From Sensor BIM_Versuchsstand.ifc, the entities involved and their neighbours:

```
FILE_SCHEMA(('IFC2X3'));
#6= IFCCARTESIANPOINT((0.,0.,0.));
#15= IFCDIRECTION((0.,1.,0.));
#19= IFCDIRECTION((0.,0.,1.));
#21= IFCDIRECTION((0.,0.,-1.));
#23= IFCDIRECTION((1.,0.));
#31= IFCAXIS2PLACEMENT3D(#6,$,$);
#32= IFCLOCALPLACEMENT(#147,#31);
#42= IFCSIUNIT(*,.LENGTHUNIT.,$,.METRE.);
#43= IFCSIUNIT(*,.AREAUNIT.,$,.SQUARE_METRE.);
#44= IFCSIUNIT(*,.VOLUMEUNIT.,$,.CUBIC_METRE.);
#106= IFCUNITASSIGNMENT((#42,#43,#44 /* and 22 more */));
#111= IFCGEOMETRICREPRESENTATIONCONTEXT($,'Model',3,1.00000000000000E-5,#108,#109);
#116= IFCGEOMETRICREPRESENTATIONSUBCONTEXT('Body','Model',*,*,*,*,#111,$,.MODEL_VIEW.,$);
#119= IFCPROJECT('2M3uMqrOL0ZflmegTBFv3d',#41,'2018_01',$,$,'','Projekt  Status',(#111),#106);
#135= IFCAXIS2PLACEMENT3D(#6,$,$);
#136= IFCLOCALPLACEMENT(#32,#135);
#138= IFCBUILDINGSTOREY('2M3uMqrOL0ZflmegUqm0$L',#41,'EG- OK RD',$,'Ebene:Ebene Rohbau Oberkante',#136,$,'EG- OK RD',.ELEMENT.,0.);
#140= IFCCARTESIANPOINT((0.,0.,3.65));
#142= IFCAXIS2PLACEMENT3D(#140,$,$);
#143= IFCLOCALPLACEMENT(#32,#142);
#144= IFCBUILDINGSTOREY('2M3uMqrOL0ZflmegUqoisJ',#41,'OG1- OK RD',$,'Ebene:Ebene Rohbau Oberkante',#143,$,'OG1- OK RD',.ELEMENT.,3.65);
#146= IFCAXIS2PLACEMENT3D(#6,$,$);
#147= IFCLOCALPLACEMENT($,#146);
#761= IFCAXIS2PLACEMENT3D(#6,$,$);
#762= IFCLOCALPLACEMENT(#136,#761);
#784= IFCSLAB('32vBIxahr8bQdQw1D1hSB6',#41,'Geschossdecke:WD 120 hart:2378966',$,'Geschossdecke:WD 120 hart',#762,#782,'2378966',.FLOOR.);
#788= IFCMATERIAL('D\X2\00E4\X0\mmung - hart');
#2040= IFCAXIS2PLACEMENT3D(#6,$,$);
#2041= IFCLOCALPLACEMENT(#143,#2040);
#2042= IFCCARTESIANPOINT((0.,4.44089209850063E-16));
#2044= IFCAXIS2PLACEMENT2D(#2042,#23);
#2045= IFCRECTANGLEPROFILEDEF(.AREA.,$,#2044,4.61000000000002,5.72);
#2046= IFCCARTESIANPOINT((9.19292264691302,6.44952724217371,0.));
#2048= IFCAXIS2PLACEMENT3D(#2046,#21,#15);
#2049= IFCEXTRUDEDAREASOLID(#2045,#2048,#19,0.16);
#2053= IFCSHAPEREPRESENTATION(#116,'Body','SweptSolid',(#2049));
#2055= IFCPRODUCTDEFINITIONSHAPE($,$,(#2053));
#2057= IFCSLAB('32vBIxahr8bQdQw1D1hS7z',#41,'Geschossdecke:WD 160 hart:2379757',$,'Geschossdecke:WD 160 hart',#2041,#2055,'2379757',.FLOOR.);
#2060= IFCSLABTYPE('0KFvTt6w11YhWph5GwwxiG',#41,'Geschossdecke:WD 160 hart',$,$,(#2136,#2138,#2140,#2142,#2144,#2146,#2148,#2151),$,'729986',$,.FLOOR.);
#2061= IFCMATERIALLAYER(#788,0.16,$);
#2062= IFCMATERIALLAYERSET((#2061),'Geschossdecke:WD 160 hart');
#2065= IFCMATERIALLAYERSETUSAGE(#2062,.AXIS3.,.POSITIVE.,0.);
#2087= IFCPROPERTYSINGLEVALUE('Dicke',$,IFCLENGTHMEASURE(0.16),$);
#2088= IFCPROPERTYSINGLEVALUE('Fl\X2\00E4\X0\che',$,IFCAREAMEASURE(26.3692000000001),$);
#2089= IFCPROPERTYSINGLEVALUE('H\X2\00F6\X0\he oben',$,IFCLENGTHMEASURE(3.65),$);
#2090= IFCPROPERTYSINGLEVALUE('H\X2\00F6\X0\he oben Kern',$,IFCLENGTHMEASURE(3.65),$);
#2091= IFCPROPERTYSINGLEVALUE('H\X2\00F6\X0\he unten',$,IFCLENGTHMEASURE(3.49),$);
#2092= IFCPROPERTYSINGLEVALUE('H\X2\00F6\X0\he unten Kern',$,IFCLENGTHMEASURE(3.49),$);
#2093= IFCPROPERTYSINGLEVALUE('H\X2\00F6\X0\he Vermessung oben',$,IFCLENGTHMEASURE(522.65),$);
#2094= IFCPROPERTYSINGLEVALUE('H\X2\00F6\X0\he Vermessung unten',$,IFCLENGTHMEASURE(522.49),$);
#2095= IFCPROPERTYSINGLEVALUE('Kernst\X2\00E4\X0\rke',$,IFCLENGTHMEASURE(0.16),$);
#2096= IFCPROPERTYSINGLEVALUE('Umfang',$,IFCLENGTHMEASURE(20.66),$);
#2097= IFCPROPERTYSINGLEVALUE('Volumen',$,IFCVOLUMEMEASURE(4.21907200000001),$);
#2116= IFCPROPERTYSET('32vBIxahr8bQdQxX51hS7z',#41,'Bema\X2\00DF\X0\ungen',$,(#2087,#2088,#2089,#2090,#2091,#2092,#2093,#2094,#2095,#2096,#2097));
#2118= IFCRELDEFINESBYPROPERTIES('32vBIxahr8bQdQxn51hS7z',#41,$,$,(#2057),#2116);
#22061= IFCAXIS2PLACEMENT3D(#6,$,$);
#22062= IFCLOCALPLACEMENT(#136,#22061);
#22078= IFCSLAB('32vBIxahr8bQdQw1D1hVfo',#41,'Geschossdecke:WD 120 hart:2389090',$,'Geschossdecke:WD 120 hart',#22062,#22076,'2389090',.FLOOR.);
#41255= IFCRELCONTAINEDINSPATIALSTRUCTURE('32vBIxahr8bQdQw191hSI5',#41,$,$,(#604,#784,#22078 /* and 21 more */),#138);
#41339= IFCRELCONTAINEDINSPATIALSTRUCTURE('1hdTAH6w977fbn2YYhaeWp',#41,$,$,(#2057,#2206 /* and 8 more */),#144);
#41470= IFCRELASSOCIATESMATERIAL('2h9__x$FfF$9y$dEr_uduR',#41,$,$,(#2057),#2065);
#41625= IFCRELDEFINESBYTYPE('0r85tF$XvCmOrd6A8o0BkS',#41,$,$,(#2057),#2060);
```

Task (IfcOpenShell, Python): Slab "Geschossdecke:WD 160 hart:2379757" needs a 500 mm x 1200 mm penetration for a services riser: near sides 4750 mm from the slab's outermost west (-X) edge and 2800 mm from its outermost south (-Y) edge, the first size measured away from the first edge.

```python
import numpy as np
import ifcopenshell
import ifcopenshell.api.feature
import ifcopenshell.api.geometry
import ifcopenshell.api.pset
import ifcopenshell.api.root
import ifcopenshell.geom
import ifcopenshell.util.element
import ifcopenshell.util.placement
import ifcopenshell.util.representation
import ifcopenshell.util.shape
import ifcopenshell.util.unit

model = ifcopenshell.open("Sensor BIM_Versuchsstand.ifc")
unit_scale = ifcopenshell.util.unit.calculate_unit_scale(model)
area_scale = ifcopenshell.util.unit.calculate_unit_scale(model, "AREAUNIT")
volume_scale = ifcopenshell.util.unit.calculate_unit_scale(model, "VOLUMEUNIT")
settings = ifcopenshell.geom.settings()


def volume(element):
    """Net volume in cubic metres, openings subtracted."""
    shape = ifcopenshell.geom.create_shape(settings, element)
    return ifcopenshell.util.shape.get_volume(shape.geometry)


slab = model.by_guid("32vBIxahr8bQdQw1D1hS7z")
before = volume(slab)

# Extent in the slab's own axes, in metres. The edges named are its -X and -Y sides.
slab_shape = ifcopenshell.geom.create_shape(settings, slab)
vertices = ifcopenshell.util.shape.get_vertices(slab_shape.geometry)
x_min, y_min, bottom = vertices.min(axis=0)
top = vertices[:, 2].max()

opening = ifcopenshell.api.root.create_entity(model, ifc_class="IfcOpeningElement", name="Services riser opening")
context = ifcopenshell.util.representation.get_context(model, "Model", "Body", "MODEL_VIEW")
width, depth = 0.5, 1.2
outline = [(0.0, 0.0), (width, 0.0), (width, depth), (0.0, depth), (0.0, 0.0)]
# Overshoot both faces by 50 mm so the cut is clean.
shape = ifcopenshell.api.geometry.add_slab_representation(
    model, context=context, depth=top - bottom + 0.1, polyline=outline
)
ifcopenshell.api.geometry.assign_representation(model, product=opening, representation=shape)

matrix = ifcopenshell.util.placement.get_local_placement(slab.ObjectPlacement)
matrix[:, 3] = matrix @ np.append(np.array([x_min + 4.75, y_min + 2.8, bottom - 0.05]) / unit_scale, 1.0)
ifcopenshell.api.geometry.edit_object_placement(model, product=opening, matrix=matrix, is_si=False)
ifcopenshell.api.feature.add_feature(model, feature=opening, element=slab)

after = volume(slab)

# Update the slab's stored quantities.
pset = model.by_id(ifcopenshell.util.element.get_pset(slab, "Bemaßungen", should_inherit=False)["id"])
ifcopenshell.api.pset.edit_pset(model, pset=pset, properties={
    "Fläche": model.create_entity("IfcAreaMeasure", after / (top - bottom) / area_scale),
    "Volumen": model.create_entity("IfcVolumeMeasure", after / volume_scale),
})

print(f"slab volume {before:.3f} -> {after:.3f} m3")

model.write("Sensor BIM_Versuchsstand_v2.ifc")
```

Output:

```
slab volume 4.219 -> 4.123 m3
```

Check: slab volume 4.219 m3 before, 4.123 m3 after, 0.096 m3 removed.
